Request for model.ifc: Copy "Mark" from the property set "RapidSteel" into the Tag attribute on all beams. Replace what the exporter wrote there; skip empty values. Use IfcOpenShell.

First a look at what the model holds.

```python
import ifcopenshell
import ifcopenshell.util.element

model = ifcopenshell.open("model.ifc")
print(model.schema)
beams = model.by_type("IfcBeam")
print(len(beams), "beams")
for e in beams[:8]:
    source = ifcopenshell.util.element.get_pset(e, "RapidSteel", "Mark")
    target = e.Tag
    print(e.id(), repr(source), repr(target), sep=" | ")
```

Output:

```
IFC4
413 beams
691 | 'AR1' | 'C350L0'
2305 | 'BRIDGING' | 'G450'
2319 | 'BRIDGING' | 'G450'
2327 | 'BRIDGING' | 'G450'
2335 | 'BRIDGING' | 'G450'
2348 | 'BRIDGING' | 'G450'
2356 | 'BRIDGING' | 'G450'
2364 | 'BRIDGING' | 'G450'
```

```python
import ifcopenshell
import ifcopenshell.util.element

model = ifcopenshell.open("model.ifc")

count = 0
for e in model.by_type("IfcBeam"):
    value = ifcopenshell.util.element.get_pset(e, "RapidSteel", "Mark")
    current = e.Tag
    if not value or not value.strip() or current == value:
        continue
    e.Tag = value
    count += 1

print(count, "beams updated")

model.write("model-out.ifc")
```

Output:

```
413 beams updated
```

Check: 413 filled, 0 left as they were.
